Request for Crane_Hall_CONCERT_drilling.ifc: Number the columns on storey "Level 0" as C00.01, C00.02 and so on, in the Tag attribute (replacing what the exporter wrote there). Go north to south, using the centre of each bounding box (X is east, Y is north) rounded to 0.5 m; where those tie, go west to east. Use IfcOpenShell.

First a look at what the model holds.

```python
import ifcopenshell
import ifcopenshell.util.element
import ifcopenshell.util.placement

model = ifcopenshell.open("Crane_Hall_CONCERT_drilling.ifc")
print(model.schema)
storey = next(s for s in model.by_type("IfcBuildingStorey") if s.Name == "Level 0")
columns = [e for e in ifcopenshell.util.element.get_decomposition(storey) if e.is_a("IfcColumn")]
for e in sorted(columns, key=lambda e: e.id()):
    origin = ifcopenshell.util.placement.get_local_placement(e.ObjectPlacement)[:3, 3]
    print(e.id(), e.Tag, e.Name, origin.round(2) + 0.0, sep=" | ")
```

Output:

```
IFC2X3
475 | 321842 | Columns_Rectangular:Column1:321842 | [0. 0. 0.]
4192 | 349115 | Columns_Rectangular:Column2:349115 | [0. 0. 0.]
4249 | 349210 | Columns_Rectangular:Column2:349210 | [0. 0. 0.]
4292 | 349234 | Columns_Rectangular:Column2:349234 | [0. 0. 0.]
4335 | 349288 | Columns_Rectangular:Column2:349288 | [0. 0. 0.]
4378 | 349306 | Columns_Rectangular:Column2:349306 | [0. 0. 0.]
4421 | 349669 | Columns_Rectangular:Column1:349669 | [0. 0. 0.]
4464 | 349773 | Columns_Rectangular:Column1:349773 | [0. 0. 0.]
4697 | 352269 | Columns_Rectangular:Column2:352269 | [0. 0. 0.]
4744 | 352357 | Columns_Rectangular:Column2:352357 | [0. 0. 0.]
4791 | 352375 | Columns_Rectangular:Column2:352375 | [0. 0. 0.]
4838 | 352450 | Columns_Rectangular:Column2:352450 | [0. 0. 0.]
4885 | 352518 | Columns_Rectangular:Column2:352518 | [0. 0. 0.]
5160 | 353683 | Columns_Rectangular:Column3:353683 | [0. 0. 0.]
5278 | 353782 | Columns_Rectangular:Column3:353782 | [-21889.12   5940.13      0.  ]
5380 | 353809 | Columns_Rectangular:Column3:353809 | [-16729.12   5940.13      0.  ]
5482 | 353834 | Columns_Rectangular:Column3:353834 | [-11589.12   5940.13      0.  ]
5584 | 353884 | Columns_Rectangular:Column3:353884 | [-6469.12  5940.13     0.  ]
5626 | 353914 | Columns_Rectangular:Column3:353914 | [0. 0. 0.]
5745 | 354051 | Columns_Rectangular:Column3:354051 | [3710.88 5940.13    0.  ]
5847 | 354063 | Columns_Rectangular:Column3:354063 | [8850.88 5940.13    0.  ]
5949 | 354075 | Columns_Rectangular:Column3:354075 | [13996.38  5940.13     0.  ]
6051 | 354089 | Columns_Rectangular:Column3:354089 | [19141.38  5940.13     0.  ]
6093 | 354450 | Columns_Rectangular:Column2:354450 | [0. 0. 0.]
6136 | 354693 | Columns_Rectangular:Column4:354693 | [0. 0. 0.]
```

```python
import ifcopenshell
import ifcopenshell.geom
import ifcopenshell.util.element
import ifcopenshell.util.shape

model = ifcopenshell.open("Crane_Hall_CONCERT_drilling.ifc")
settings = ifcopenshell.geom.settings()
settings.set("use-world-coords", True)


def centre(element):
    shape = ifcopenshell.geom.create_shape(settings, element)
    return ifcopenshell.util.shape.get_bbox_centroid(shape.geometry)


storey = next(s for s in model.by_type("IfcBuildingStorey") if s.Name == "Level 0")
columns = [e for e in ifcopenshell.util.element.get_decomposition(storey) if e.is_a("IfcColumn")]

# Insertion points can sit at a corner or the storey origin, so sort by the geometry (in metres).
centres = {e: centre(e) for e in columns}
columns.sort(key=lambda e: (-round(centres[e][1] / 0.5), centres[e][0]))

for i, e in enumerate(columns, start=1):
    number = f"C00.{i:02d}"
    e.Tag = number
    print(e.id(), number)

model.write("Crane_Hall_CONCERT_drilling_updated.ifc")
```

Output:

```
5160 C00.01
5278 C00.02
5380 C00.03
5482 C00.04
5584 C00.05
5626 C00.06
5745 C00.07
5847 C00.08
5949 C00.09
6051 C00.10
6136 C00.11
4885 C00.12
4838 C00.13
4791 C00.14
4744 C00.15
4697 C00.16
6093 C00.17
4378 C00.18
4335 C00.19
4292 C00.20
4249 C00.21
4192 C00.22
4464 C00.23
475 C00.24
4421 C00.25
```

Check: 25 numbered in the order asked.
